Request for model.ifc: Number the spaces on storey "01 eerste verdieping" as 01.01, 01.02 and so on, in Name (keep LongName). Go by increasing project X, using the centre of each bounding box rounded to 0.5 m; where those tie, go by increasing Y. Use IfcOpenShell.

First a look at what the model holds.

```python
import ifcopenshell
import ifcopenshell.util.element
import ifcopenshell.util.placement

model = ifcopenshell.open("model.ifc")
print(model.schema)
storey = next(s for s in model.by_type("IfcBuildingStorey") if s.Name == "01 eerste verdieping")
spaces = [e for e in ifcopenshell.util.element.get_decomposition(storey) if e.is_a("IfcSpace")]
for e in sorted(spaces, key=lambda e: e.id()):
    origin = ifcopenshell.util.placement.get_local_placement(e.ObjectPlacement)[:3, 3]
    print(e.id(), e.Name, e.LongName, origin.round(2) + 0.0, sep=" | ")
```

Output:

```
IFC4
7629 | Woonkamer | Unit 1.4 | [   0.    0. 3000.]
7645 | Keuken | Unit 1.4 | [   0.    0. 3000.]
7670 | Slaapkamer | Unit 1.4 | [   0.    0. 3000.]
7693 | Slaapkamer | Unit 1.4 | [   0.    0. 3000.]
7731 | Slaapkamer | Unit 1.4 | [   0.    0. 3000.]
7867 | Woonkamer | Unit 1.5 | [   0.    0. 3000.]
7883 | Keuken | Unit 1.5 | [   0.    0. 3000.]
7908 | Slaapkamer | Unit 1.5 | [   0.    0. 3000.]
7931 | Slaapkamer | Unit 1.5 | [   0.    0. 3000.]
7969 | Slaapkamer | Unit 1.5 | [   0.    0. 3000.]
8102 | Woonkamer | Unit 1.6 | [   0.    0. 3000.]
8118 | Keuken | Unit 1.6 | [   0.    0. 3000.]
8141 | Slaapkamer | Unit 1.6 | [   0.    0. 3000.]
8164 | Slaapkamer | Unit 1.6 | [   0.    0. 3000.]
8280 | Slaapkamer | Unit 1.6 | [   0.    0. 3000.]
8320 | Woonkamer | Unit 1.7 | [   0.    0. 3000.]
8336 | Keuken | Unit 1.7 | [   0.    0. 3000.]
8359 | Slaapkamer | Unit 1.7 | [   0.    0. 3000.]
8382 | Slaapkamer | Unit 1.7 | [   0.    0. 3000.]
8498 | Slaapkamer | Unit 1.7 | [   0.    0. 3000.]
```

```python
import ifcopenshell
import ifcopenshell.geom
import ifcopenshell.util.element
import ifcopenshell.util.shape

model = ifcopenshell.open("model.ifc")
settings = ifcopenshell.geom.settings()
settings.set("use-world-coords", True)


def centre(element):
    shape = ifcopenshell.geom.create_shape(settings, element)
    return ifcopenshell.util.shape.get_bbox_centroid(shape.geometry)


storey = next(s for s in model.by_type("IfcBuildingStorey") if s.Name == "01 eerste verdieping")
spaces = [e for e in ifcopenshell.util.element.get_decomposition(storey) if e.is_a("IfcSpace")]

# Insertion points can sit at a corner or the storey origin, so sort by the geometry (in metres).
centres = {e: centre(e) for e in spaces}
spaces.sort(key=lambda e: (round(centres[e][0] / 0.5), centres[e][1]))

for i, e in enumerate(spaces, start=1):
    number = f"01.{i:02d}"
    e.Name = number
    print(e.id(), number)

model.write("model-out.ifc")
```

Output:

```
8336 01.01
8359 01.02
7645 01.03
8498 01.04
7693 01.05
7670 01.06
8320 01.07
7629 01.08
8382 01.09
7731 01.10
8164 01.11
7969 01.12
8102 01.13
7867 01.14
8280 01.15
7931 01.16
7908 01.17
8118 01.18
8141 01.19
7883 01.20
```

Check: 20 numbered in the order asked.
